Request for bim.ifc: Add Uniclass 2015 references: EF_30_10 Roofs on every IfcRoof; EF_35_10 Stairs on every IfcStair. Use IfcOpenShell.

First a look at what the model holds.

```python
import ifcopenshell

model = ifcopenshell.open("bim.ifc")
print(model.schema)
print("classifications:", [c.Name for c in model.by_type("IfcClassification")])
for ifc_class in ("IfcDoor", "IfcRoof", "IfcStair", "IfcWall", "IfcWindow"):
    print(ifc_class, len(model.by_type(ifc_class)))
```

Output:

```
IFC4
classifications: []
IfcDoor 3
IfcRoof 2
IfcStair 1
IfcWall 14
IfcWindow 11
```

```python
import ifcopenshell
import ifcopenshell.api.classification

model = ifcopenshell.open("bim.ifc")

system = ifcopenshell.api.classification.add_classification(model, classification="Uniclass 2015")

codes = {
    "IfcRoof": ("EF_30_10", "Roofs"),
    "IfcStair": ("EF_35_10", "Stairs"),
}
for ifc_class, (code, name) in codes.items():
    products = model.by_type(ifc_class)
    ifcopenshell.api.classification.add_reference(
        model, products=products, classification=system, identification=code, name=name
    )
    print(code, len(products))

model.write("bim_v2.ifc")
```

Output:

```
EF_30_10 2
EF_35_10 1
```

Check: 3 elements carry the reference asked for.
